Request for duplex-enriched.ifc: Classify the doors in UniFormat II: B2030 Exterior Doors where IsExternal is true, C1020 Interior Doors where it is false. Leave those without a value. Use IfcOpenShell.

First a look at what the model holds.

```python
import ifcopenshell
import ifcopenshell.util.element

model = ifcopenshell.open("duplex-enriched.ifc")
print(model.schema)
print("classifications:", [c.Name for c in model.by_type("IfcClassification")])
values = [ifcopenshell.util.element.get_pset(e, "Pset_DoorCommon", "IsExternal") for e in model.by_type("IfcDoor")]
for value in (True, False, None):
    print("IsExternal", value, values.count(value))
```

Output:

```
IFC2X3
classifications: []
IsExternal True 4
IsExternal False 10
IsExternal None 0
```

```python
import ifcopenshell
import ifcopenshell.api.classification
import ifcopenshell.util.element

model = ifcopenshell.open("duplex-enriched.ifc")

# IFC2X3 requires Source and Edition and has no link from the project to the system.
system = model.create_entity("IfcClassification", Source="ASTM", Edition="E1557", Name="UniFormat II")

doors = model.by_type("IfcDoor")
external = {e: ifcopenshell.util.element.get_pset(e, "Pset_DoorCommon", "IsExternal") for e in doors}
for flag, code, name in ((True, "B2030", "Exterior Doors"), (False, "C1020", "Interior Doors")):
    products = [e for e in doors if external[e] is flag]
    ifcopenshell.api.classification.add_reference(
        model, products=products, classification=system, identification=code, name=name
    )
    print(code, len(products))

model.write("duplex-enriched-out.ifc")
```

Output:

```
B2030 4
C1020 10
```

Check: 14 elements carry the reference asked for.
